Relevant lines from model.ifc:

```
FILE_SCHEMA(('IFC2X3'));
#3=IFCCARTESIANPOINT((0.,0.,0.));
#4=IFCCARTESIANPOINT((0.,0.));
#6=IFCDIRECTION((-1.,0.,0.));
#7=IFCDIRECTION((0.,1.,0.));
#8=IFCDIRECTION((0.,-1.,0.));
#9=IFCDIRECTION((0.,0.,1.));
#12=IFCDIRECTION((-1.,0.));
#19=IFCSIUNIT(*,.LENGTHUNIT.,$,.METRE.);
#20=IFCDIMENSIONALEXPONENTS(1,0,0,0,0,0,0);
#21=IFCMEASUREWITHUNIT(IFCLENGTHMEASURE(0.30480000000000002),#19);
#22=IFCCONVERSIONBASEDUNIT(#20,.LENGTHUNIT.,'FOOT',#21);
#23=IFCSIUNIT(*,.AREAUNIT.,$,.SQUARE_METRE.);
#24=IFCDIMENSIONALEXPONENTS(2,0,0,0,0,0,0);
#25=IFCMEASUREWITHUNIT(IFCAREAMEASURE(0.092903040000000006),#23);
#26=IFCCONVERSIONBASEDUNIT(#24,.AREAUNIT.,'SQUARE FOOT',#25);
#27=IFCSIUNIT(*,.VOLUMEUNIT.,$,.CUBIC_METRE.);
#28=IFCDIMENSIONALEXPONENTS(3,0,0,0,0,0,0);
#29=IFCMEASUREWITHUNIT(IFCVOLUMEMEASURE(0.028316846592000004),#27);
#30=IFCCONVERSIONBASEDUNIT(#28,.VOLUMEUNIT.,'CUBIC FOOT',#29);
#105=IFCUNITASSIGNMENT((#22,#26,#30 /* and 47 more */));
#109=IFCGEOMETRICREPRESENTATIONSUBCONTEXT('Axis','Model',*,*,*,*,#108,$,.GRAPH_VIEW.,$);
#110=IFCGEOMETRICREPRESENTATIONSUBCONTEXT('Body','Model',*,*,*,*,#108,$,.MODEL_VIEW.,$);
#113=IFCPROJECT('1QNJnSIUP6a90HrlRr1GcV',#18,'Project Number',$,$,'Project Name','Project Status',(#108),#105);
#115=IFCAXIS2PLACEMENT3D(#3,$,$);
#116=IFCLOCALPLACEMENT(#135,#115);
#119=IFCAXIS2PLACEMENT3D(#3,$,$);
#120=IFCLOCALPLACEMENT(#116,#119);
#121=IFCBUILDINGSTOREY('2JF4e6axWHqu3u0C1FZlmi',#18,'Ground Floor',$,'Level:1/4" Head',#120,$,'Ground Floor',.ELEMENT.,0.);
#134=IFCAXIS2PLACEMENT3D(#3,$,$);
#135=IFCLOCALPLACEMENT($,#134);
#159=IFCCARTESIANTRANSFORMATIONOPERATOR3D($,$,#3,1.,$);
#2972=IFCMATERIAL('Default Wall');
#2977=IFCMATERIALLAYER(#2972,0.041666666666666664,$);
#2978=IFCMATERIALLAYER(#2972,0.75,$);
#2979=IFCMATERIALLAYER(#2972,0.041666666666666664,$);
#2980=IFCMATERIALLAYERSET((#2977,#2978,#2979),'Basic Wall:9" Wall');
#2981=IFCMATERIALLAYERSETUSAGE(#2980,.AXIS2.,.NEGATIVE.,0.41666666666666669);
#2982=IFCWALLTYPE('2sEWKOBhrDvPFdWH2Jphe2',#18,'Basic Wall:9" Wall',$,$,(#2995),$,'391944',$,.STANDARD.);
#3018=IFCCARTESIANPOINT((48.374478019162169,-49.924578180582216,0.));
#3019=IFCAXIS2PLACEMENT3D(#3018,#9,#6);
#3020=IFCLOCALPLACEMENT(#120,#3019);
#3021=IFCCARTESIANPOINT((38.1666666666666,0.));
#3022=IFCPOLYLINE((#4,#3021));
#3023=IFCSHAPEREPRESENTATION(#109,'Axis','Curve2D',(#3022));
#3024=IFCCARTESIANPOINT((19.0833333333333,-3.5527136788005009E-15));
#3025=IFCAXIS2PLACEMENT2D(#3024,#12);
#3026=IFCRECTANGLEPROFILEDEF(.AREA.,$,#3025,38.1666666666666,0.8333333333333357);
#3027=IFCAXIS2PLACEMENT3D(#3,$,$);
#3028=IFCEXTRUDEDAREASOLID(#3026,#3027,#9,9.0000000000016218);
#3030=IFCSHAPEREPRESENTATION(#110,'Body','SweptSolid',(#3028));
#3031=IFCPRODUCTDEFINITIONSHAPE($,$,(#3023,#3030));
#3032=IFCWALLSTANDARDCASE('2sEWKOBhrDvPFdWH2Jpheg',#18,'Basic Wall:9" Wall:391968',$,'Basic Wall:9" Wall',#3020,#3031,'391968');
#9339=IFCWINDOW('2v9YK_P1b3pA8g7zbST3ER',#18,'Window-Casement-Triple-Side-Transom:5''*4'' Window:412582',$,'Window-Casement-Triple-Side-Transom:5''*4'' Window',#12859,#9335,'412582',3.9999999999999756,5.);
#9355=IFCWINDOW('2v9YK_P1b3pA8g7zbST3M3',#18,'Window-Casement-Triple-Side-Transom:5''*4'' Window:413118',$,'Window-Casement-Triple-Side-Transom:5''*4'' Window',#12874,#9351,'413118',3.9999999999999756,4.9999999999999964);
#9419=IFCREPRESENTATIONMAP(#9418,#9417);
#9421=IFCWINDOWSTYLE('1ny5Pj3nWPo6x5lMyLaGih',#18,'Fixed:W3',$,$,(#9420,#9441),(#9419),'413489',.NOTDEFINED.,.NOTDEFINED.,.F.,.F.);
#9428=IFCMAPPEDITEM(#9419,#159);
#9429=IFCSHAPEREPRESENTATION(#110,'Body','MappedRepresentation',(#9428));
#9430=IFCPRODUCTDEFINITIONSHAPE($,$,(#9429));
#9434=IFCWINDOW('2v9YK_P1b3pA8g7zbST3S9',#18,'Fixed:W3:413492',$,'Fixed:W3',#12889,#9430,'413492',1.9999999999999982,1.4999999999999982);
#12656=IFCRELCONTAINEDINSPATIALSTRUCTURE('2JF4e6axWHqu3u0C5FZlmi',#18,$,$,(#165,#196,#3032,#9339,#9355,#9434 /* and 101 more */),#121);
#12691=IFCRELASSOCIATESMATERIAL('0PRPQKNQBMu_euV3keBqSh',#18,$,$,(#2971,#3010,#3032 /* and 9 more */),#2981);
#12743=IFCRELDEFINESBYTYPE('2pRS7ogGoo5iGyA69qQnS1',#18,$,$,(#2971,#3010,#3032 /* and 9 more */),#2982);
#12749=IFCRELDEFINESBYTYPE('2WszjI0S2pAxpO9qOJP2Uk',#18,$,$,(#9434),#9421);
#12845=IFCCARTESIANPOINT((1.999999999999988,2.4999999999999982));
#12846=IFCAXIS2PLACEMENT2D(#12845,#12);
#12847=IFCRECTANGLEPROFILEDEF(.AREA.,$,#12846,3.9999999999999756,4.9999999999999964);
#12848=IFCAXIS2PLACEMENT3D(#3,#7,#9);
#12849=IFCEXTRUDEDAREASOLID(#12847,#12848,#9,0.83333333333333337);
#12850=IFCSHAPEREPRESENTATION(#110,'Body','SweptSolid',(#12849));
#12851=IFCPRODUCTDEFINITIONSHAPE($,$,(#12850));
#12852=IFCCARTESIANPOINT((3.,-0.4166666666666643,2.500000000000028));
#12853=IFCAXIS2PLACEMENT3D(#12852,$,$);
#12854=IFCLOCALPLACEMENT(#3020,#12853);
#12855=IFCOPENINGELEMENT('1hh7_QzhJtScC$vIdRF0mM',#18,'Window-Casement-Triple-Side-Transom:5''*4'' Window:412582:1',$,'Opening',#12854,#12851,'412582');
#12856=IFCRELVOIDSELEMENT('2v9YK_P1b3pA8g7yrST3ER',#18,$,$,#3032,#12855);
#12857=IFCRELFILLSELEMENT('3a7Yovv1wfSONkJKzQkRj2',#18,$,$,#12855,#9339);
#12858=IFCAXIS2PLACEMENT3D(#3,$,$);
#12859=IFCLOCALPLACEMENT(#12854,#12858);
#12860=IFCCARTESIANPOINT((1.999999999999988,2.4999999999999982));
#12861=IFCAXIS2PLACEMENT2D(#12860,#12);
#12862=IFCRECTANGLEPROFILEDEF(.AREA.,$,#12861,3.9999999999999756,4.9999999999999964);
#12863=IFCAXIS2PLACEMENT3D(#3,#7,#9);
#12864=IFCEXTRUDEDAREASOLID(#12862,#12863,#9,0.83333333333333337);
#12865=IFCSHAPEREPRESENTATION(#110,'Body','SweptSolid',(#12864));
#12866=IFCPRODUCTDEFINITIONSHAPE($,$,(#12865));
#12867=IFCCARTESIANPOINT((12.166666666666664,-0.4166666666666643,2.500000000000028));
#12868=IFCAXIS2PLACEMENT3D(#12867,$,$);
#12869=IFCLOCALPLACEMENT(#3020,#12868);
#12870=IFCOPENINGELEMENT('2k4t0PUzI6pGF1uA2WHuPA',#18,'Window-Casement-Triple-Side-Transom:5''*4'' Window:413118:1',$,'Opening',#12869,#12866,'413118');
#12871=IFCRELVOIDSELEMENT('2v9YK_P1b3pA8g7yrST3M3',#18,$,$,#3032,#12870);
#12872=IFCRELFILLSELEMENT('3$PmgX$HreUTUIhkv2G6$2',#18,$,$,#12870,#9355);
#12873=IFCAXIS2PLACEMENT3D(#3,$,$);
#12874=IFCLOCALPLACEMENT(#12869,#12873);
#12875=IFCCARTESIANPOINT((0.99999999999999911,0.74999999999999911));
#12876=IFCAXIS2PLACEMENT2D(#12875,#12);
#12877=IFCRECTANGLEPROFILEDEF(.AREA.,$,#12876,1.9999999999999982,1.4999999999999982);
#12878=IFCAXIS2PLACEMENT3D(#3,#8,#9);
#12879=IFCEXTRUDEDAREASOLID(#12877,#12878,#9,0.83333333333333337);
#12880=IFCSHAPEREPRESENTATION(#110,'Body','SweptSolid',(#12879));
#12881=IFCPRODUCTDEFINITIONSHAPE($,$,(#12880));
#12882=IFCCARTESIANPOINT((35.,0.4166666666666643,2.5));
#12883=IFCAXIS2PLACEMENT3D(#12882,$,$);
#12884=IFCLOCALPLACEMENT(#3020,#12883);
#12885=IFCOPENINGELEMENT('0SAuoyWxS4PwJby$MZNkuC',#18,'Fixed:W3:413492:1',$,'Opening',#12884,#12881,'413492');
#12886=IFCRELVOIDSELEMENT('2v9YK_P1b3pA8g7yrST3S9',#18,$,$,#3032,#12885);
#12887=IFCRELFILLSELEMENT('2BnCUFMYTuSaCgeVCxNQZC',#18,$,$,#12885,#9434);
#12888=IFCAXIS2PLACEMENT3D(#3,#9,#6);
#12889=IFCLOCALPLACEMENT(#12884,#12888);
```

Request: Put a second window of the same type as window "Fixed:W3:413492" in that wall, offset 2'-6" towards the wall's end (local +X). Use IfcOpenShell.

```python
import ifcopenshell
import ifcopenshell.api.feature
import ifcopenshell.api.geometry
import ifcopenshell.api.root
import ifcopenshell.geom
import ifcopenshell.util.element
import ifcopenshell.util.placement
import ifcopenshell.util.shape
import ifcopenshell.util.unit

model = ifcopenshell.open("model.ifc")
unit_scale = ifcopenshell.util.unit.calculate_unit_scale(model)
settings = ifcopenshell.geom.settings()


def volume(element):
    """Net volume in cubic metres, openings subtracted."""
    shape = ifcopenshell.geom.create_shape(settings, element)
    return ifcopenshell.util.shape.get_volume(shape.geometry)


def reuse_history(source, copy):
    """copy_class also copies each property set's owner history, people and application; keep the originals."""
    for rel in copy.IsDefinedBy:
        if rel.is_a("IfcRelDefinesByProperties") and (history := rel.RelatingPropertyDefinition.OwnerHistory):
            rel.RelatingPropertyDefinition.OwnerHistory = source.OwnerHistory
            ifcopenshell.util.element.remove_deep2(model, history)


window = model.by_id(9434)
opening = window.FillsVoids[0].RelatingOpeningElement
wall = opening.VoidsElements[0].RelatingBuildingElement
before = volume(wall)
shift = ifcopenshell.util.placement.get_local_placement(wall.ObjectPlacement)[:3, 0] * 30 * 0.0254 / unit_scale

# copy_class copies the void relationship, type, container and properties, but no geometry.
new_opening = ifcopenshell.api.root.copy_class(model, product=opening)
new_opening.Representation = ifcopenshell.util.element.copy_deep(
    model, opening.Representation, exclude=["IfcGeometricRepresentationContext", "IfcRepresentationMap"]
)
new_opening.Name = "Fixed:W3"
new_opening.Tag = None
new_window = ifcopenshell.api.root.copy_class(model, product=window)
new_window.Representation = ifcopenshell.util.element.copy_deep(
    model, window.Representation, exclude=["IfcGeometricRepresentationContext", "IfcRepresentationMap"]
)
new_window.Name = "Fixed:W3"
new_window.Tag = None
reuse_history(window, new_window)
fills = ifcopenshell.api.feature.add_filling(model, opening=new_opening, element=new_window)
fills.OwnerHistory = new_window.OwnerHistory  # required in IFC2X3

for old, new in ((opening, new_opening), (window, new_window)):
    matrix = ifcopenshell.util.placement.get_local_placement(old.ObjectPlacement)
    matrix[:3, 3] += shift
    ifcopenshell.api.geometry.edit_object_placement(model, product=new, matrix=matrix, is_si=False)

after = volume(wall)

print(f"wall volume {before:.3f} -> {after:.3f} m3")

model.write("model_rev.ifc")
```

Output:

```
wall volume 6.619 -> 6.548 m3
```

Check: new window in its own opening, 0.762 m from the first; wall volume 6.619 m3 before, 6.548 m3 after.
